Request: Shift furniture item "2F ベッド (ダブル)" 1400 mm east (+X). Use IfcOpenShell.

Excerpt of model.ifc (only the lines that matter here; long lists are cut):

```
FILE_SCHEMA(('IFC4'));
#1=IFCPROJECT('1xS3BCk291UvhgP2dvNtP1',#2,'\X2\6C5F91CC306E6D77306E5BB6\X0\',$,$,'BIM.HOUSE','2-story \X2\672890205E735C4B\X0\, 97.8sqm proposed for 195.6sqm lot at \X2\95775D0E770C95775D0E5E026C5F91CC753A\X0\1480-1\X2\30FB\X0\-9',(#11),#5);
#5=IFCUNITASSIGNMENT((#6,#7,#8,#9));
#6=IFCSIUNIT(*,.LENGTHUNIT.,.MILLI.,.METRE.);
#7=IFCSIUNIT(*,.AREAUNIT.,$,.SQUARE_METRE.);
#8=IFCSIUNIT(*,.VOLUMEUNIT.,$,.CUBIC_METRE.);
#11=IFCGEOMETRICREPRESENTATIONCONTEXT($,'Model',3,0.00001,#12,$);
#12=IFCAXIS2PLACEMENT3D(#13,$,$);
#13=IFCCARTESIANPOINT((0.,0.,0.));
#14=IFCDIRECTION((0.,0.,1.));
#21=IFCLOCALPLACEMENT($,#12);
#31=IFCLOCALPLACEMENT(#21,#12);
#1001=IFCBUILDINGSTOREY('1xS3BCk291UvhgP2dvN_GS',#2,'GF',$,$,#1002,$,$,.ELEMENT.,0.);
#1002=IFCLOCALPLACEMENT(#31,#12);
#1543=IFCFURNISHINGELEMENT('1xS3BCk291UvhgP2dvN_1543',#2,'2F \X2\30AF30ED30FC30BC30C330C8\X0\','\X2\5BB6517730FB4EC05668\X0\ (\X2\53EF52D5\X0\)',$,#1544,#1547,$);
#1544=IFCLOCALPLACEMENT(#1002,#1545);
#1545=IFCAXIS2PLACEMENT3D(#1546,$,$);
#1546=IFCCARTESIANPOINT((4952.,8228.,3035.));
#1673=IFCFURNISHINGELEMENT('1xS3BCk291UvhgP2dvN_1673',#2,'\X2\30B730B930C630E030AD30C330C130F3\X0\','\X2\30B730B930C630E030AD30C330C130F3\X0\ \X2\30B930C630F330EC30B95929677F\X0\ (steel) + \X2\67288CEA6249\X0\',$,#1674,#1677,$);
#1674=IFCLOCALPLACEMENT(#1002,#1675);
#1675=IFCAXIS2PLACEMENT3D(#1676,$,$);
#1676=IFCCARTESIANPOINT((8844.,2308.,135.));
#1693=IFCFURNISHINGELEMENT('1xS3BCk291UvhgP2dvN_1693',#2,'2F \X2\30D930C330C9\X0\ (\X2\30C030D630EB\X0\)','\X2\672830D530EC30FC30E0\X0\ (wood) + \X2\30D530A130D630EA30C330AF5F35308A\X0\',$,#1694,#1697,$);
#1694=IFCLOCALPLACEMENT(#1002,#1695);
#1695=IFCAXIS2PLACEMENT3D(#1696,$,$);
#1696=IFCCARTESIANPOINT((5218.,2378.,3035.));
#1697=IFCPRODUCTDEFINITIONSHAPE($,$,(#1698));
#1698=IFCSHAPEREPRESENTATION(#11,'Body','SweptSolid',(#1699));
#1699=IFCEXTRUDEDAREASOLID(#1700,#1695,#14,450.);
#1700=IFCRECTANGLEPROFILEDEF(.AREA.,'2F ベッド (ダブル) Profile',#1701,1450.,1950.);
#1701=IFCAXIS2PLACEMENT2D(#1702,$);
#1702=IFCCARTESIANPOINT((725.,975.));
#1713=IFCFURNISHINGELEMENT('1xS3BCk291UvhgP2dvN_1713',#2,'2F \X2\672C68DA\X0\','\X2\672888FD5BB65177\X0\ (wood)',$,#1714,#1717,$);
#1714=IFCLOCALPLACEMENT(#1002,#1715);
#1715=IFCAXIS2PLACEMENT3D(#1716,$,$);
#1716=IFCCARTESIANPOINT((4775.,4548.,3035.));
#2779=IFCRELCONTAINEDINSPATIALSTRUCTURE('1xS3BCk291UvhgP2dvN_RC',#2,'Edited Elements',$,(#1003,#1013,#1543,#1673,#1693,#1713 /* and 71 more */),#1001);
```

```python
import ifcopenshell
import ifcopenshell.api.geometry
import ifcopenshell.util.placement

model = ifcopenshell.open("model.ifc")

item = model.by_id(1693)
matrix = ifcopenshell.util.placement.get_local_placement(item.ObjectPlacement)
matrix[0, 3] += 1400.0
ifcopenshell.api.geometry.edit_object_placement(model, product=item, matrix=matrix, is_si=False)

print(ifcopenshell.util.placement.get_local_placement(item.ObjectPlacement).round(3) + 0.0)

model.write("model-out.ifc")
```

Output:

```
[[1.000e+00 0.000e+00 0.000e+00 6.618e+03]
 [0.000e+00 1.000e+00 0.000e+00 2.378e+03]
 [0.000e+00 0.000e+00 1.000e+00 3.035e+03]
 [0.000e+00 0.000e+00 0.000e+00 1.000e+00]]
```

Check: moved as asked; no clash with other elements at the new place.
